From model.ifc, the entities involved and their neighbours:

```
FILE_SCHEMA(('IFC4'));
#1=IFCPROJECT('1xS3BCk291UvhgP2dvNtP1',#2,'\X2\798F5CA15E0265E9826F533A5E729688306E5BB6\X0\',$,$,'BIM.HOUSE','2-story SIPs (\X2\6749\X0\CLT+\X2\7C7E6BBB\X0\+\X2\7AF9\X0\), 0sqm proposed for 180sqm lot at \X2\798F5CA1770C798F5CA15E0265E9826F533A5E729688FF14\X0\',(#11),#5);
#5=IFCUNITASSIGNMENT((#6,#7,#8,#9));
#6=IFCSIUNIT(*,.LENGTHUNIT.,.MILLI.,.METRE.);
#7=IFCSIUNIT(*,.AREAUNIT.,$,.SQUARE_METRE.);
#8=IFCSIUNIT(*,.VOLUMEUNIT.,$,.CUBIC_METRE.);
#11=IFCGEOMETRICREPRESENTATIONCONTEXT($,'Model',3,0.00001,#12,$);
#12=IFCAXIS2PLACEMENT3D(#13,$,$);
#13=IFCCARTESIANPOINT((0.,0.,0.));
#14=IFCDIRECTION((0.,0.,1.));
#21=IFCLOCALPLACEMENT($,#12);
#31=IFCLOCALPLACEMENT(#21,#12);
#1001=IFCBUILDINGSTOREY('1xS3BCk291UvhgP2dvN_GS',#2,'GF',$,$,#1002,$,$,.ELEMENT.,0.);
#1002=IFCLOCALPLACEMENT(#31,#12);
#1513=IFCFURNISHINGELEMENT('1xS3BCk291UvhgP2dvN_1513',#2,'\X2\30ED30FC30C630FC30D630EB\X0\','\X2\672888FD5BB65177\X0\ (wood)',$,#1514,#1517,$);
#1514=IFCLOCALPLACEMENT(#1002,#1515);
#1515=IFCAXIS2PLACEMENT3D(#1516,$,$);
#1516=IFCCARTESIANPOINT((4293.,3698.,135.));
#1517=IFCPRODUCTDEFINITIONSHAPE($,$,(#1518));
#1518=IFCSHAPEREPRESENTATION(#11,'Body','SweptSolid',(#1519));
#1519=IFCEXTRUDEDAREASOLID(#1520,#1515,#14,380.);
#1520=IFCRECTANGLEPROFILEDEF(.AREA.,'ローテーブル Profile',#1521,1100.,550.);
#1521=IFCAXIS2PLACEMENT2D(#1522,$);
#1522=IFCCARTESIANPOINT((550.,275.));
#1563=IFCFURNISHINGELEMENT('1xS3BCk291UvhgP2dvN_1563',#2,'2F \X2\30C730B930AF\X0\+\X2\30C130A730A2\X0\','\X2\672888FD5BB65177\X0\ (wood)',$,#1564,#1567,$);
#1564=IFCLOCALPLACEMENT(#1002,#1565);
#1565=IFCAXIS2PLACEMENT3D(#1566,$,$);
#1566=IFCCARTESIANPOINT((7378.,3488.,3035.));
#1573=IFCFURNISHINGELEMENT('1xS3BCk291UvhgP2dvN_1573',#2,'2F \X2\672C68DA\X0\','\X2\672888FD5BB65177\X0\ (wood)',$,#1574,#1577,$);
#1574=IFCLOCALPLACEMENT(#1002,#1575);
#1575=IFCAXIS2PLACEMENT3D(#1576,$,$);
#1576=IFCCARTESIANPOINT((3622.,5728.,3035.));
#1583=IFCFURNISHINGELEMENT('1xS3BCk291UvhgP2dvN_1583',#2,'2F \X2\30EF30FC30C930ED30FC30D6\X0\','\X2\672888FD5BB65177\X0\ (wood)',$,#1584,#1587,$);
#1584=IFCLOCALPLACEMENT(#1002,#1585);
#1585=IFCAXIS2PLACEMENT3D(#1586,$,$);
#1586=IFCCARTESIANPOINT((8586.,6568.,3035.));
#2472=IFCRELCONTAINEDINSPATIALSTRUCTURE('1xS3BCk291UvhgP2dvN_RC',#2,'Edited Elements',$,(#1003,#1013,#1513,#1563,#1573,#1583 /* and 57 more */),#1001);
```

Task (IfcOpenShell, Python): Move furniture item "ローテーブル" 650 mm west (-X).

```python
import ifcopenshell
import ifcopenshell.api.geometry
import ifcopenshell.util.placement
import ifcopenshell.util.unit

model = ifcopenshell.open("model.ifc")
unit_scale = ifcopenshell.util.unit.calculate_unit_scale(model)

item = model.by_guid("1xS3BCk291UvhgP2dvN_1513")
matrix = ifcopenshell.util.placement.get_local_placement(item.ObjectPlacement)
matrix[0, 3] -= 0.65 / unit_scale
ifcopenshell.api.geometry.edit_object_placement(model, product=item, matrix=matrix, is_si=False)

print(ifcopenshell.util.placement.get_local_placement(item.ObjectPlacement).round(3) + 0.0)

model.write("model_v2.ifc")
```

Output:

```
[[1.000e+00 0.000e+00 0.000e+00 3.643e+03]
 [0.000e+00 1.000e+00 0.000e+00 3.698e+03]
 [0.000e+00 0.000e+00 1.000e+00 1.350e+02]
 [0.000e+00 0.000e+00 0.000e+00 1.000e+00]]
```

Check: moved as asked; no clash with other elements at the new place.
